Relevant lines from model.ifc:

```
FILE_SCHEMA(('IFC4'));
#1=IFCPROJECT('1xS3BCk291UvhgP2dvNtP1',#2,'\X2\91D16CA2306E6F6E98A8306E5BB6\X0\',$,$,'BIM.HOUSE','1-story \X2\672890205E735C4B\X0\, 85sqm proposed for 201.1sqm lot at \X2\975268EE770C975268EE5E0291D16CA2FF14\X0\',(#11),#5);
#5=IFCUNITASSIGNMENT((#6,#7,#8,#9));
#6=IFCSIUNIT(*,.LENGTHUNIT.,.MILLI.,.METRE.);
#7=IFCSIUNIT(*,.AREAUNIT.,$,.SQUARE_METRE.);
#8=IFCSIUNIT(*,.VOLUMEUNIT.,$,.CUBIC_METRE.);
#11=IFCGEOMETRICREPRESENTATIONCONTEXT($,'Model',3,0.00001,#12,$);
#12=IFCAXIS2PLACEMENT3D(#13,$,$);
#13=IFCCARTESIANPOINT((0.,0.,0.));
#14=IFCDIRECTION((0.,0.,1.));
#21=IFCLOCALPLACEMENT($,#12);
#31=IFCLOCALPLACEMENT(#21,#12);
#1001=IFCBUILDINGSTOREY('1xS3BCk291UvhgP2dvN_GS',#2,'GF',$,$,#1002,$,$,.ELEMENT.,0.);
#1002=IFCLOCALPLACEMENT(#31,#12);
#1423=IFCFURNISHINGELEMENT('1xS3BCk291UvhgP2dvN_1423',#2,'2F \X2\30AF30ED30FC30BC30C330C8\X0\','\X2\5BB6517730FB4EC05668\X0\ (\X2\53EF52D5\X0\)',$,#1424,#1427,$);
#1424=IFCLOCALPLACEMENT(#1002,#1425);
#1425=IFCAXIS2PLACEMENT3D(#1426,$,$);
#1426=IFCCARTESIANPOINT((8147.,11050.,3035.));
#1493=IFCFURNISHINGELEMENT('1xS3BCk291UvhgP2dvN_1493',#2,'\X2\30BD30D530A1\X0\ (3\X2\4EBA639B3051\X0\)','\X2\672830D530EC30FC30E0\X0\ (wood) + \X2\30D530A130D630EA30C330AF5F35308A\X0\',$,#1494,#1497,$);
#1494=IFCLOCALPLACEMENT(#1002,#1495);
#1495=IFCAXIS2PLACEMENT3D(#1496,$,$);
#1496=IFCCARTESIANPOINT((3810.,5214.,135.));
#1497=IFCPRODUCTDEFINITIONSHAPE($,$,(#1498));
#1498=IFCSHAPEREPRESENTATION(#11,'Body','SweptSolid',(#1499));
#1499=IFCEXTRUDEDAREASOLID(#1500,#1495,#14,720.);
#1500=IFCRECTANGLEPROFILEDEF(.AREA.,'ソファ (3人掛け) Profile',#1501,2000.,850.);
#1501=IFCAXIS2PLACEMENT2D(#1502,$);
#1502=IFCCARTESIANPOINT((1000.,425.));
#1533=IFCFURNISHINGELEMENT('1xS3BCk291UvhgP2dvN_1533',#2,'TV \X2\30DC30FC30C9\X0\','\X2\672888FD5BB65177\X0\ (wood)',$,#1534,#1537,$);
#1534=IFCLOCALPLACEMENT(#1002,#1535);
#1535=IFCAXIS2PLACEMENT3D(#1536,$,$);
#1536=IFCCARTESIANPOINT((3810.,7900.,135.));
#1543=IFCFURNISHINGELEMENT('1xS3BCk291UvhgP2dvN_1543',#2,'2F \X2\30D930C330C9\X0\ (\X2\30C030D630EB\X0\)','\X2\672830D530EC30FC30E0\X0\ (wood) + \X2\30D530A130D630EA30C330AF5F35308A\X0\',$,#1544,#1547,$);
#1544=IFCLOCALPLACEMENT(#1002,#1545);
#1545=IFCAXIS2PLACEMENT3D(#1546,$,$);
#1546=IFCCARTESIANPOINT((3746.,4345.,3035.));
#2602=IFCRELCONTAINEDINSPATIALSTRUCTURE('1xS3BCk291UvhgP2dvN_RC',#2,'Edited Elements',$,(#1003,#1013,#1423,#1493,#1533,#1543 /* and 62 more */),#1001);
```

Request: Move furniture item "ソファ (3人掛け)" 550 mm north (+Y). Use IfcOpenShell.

```python
import ifcopenshell
import ifcopenshell.api.geometry
import ifcopenshell.util.placement
import ifcopenshell.util.unit

model = ifcopenshell.open("model.ifc")
unit_scale = ifcopenshell.util.unit.calculate_unit_scale(model)

item = model.by_guid("1xS3BCk291UvhgP2dvN_1493")
matrix = ifcopenshell.util.placement.get_local_placement(item.ObjectPlacement)
matrix[1, 3] += 0.55 / unit_scale
ifcopenshell.api.geometry.edit_object_placement(model, product=item, matrix=matrix, is_si=False)

print(ifcopenshell.util.placement.get_local_placement(item.ObjectPlacement).round(3) + 0.0)

model.write("model_rev.ifc")
```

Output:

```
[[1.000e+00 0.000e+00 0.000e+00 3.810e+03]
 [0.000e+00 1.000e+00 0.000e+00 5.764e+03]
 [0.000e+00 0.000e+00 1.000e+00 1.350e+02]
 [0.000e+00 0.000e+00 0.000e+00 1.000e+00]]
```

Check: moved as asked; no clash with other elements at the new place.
